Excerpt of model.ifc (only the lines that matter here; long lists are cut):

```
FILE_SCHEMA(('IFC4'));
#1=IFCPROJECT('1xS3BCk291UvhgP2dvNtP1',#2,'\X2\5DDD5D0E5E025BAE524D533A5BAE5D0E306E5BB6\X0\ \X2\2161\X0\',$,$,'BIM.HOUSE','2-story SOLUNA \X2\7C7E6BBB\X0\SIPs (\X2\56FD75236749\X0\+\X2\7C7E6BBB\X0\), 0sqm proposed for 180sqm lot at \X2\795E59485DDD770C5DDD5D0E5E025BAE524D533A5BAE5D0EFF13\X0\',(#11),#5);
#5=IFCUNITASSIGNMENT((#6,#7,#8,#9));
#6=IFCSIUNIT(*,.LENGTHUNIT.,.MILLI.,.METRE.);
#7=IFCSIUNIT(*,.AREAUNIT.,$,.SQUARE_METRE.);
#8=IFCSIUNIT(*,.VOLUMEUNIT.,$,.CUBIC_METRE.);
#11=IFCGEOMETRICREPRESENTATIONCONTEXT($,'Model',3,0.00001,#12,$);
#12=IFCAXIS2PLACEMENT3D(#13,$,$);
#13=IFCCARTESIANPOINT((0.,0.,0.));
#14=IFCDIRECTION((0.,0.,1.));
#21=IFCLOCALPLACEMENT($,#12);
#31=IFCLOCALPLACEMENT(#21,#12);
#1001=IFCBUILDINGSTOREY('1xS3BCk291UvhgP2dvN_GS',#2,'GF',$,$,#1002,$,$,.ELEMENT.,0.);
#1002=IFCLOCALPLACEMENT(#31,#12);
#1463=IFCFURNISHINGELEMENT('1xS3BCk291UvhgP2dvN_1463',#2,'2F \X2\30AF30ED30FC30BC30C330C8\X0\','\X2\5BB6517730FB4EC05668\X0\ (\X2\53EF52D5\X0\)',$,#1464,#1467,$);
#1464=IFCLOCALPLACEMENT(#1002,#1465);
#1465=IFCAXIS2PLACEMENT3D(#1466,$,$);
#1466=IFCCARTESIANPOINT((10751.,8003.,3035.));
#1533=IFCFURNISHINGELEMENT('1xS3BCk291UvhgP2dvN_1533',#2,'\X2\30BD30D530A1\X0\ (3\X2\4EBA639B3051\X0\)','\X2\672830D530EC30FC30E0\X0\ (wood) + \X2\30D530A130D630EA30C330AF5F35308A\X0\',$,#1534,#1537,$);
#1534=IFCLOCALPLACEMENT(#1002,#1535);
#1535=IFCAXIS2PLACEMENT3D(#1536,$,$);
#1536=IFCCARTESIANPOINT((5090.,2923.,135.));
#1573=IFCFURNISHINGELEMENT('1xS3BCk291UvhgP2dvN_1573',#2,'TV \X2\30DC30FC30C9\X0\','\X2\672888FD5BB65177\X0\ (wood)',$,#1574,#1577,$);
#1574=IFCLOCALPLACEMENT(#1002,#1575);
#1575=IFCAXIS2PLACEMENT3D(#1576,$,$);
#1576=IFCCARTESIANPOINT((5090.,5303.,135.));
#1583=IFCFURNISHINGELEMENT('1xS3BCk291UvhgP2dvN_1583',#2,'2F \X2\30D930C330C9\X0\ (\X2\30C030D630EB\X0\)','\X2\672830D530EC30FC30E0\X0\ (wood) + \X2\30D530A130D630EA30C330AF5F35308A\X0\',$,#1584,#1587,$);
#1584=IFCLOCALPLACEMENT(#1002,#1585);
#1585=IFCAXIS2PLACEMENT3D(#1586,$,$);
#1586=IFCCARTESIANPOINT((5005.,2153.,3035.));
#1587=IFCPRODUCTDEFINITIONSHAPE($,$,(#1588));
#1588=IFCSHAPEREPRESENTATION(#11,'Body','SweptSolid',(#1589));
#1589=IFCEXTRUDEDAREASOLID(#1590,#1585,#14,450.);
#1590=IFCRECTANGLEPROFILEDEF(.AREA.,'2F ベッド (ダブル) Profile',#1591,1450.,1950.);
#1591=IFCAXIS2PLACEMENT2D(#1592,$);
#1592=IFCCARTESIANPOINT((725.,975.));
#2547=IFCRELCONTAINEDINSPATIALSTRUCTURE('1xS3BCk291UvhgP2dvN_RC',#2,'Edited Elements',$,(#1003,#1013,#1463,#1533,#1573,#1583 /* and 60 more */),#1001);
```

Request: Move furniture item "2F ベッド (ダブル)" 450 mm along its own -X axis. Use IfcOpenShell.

```python
import ifcopenshell
import ifcopenshell.api.geometry
import ifcopenshell.util.placement
import ifcopenshell.util.unit

model = ifcopenshell.open("model.ifc")
unit_scale = ifcopenshell.util.unit.calculate_unit_scale(model)

item = model.by_id(1583)
matrix = ifcopenshell.util.placement.get_local_placement(item.ObjectPlacement)
matrix[:3, 3] -= matrix[:3, 0] * 0.45 / unit_scale
ifcopenshell.api.geometry.edit_object_placement(model, product=item, matrix=matrix, is_si=False)

print(ifcopenshell.util.placement.get_local_placement(item.ObjectPlacement).round(3) + 0.0)

model.write("model_rev.ifc")
```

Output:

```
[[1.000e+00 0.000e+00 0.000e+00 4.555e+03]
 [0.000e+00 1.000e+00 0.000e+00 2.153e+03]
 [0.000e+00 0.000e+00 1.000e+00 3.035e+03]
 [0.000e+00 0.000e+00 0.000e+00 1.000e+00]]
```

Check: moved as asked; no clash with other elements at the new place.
